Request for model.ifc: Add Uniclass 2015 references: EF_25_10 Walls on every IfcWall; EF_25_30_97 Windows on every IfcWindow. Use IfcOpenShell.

First a look at what the model holds.

```python
import ifcopenshell

model = ifcopenshell.open("model.ifc")
print(model.schema)
print("classifications:", [c.Name for c in model.by_type("IfcClassification")])
for ifc_class in ("IfcDoor", "IfcRoof", "IfcStair", "IfcWall", "IfcWindow"):
    print(ifc_class, len(model.by_type(ifc_class)))
```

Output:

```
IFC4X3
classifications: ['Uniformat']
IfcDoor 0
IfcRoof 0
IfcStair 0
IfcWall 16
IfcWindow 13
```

```python
import ifcopenshell
import ifcopenshell.api.classification

model = ifcopenshell.open("model.ifc")

system = ifcopenshell.api.classification.add_classification(model, classification="Uniclass 2015")

codes = {
    "IfcWall": ("EF_25_10", "Walls"),
    "IfcWindow": ("EF_25_30_97", "Windows"),
}
for ifc_class, (code, name) in codes.items():
    products = model.by_type(ifc_class)
    ifcopenshell.api.classification.add_reference(
        model, products=products, classification=system, identification=code, name=name
    )
    print(code, len(products))

model.write("model_edited.ifc")
```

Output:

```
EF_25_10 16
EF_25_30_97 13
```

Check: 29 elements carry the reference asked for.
